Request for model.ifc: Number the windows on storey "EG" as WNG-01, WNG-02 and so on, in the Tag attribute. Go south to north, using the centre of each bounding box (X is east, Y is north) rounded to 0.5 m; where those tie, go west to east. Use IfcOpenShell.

First a look at what the model holds.

```python
import ifcopenshell
import ifcopenshell.util.element
import ifcopenshell.util.placement

model = ifcopenshell.open("model.ifc")
print(model.schema)
storey = next(s for s in model.by_type("IfcBuildingStorey") if s.Name == "EG")
windows = [e for e in ifcopenshell.util.element.get_decomposition(storey) if e.is_a("IfcWindow")]
for e in sorted(windows, key=lambda e: e.id()):
    origin = ifcopenshell.util.placement.get_local_placement(e.ObjectPlacement)[:3, 3]
    print(e.id(), e.Tag, e.Name, origin.round(2) + 0.0, sep=" | ")
```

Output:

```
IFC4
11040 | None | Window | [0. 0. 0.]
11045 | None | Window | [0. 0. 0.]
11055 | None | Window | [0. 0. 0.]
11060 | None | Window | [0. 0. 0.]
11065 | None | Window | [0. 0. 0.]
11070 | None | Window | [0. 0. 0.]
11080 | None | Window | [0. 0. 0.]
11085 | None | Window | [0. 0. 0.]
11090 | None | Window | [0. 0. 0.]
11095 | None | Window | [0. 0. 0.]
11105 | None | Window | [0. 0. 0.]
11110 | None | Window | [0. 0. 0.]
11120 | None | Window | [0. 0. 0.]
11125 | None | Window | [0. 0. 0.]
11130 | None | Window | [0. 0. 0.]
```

```python
import ifcopenshell
import ifcopenshell.geom
import ifcopenshell.util.element
import ifcopenshell.util.shape

model = ifcopenshell.open("model.ifc")
settings = ifcopenshell.geom.settings()
settings.set("use-world-coords", True)


def centre(element):
    shape = ifcopenshell.geom.create_shape(settings, element)
    return ifcopenshell.util.shape.get_bbox_centroid(shape.geometry)


storey = next(s for s in model.by_type("IfcBuildingStorey") if s.Name == "EG")
windows = [e for e in ifcopenshell.util.element.get_decomposition(storey) if e.is_a("IfcWindow")]

# Insertion points can sit at a corner or the storey origin, so sort by the geometry (in metres).
centres = {e: centre(e) for e in windows}
windows.sort(key=lambda e: (round(centres[e][1] / 0.5), centres[e][0]))

for i, e in enumerate(windows, start=1):
    number = f"WNG-{i:02d}"
    e.Tag = number
    print(e.id(), number)

model.write("model_v2.ifc")
```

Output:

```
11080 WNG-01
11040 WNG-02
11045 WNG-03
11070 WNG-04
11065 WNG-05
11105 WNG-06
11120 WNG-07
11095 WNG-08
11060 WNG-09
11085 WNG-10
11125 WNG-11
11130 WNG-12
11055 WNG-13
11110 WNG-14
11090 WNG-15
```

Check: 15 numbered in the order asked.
